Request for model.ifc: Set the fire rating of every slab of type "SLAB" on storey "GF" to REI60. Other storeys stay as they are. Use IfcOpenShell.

First a look at what the model holds.

```python
import ifcopenshell
import ifcopenshell.util.element

model = ifcopenshell.open("model.ifc")
print(model.schema)
storey = next(s for s in model.by_type("IfcBuildingStorey") if s.Name == "GF")
slabs = [e for e in ifcopenshell.util.element.get_decomposition(storey) if e.is_a("IfcSlab")]
seen = {}
for e in slabs:
    element_type = ifcopenshell.util.element.get_type(e)
    key = (element_type.Name if element_type != e and element_type else None, ifcopenshell.util.element.get_pset(e, "Pset_SlabCommon", "FireRating"))
    seen[key] = seen.get(key, 0) + 1
for (name, value), count in sorted(seen.items(), key=str):
    print(count, "x", name, "|", value)
```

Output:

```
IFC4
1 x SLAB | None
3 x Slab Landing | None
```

```python
import ifcopenshell
import ifcopenshell.api.pset
import ifcopenshell.util.element

model = ifcopenshell.open("model.ifc")

storey = next(s for s in model.by_type("IfcBuildingStorey") if s.Name == "GF")
slabs = [e for e in ifcopenshell.util.element.get_decomposition(storey) if e.is_a("IfcSlab")]

count = 0
for e in slabs:
    element_type = ifcopenshell.util.element.get_type(e)
    if element_type in (None, e) or element_type.Name != "SLAB":
        continue
    # add_pset returns the element's existing set when there is one.
    pset = ifcopenshell.api.pset.add_pset(model, product=e, name="Pset_SlabCommon")
    ifcopenshell.api.pset.edit_pset(model, pset=pset, properties={"FireRating": "REI60"})
    count += 1

print(count, "slabs updated")

model.write("model_rev.ifc")
```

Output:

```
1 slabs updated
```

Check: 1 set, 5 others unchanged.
